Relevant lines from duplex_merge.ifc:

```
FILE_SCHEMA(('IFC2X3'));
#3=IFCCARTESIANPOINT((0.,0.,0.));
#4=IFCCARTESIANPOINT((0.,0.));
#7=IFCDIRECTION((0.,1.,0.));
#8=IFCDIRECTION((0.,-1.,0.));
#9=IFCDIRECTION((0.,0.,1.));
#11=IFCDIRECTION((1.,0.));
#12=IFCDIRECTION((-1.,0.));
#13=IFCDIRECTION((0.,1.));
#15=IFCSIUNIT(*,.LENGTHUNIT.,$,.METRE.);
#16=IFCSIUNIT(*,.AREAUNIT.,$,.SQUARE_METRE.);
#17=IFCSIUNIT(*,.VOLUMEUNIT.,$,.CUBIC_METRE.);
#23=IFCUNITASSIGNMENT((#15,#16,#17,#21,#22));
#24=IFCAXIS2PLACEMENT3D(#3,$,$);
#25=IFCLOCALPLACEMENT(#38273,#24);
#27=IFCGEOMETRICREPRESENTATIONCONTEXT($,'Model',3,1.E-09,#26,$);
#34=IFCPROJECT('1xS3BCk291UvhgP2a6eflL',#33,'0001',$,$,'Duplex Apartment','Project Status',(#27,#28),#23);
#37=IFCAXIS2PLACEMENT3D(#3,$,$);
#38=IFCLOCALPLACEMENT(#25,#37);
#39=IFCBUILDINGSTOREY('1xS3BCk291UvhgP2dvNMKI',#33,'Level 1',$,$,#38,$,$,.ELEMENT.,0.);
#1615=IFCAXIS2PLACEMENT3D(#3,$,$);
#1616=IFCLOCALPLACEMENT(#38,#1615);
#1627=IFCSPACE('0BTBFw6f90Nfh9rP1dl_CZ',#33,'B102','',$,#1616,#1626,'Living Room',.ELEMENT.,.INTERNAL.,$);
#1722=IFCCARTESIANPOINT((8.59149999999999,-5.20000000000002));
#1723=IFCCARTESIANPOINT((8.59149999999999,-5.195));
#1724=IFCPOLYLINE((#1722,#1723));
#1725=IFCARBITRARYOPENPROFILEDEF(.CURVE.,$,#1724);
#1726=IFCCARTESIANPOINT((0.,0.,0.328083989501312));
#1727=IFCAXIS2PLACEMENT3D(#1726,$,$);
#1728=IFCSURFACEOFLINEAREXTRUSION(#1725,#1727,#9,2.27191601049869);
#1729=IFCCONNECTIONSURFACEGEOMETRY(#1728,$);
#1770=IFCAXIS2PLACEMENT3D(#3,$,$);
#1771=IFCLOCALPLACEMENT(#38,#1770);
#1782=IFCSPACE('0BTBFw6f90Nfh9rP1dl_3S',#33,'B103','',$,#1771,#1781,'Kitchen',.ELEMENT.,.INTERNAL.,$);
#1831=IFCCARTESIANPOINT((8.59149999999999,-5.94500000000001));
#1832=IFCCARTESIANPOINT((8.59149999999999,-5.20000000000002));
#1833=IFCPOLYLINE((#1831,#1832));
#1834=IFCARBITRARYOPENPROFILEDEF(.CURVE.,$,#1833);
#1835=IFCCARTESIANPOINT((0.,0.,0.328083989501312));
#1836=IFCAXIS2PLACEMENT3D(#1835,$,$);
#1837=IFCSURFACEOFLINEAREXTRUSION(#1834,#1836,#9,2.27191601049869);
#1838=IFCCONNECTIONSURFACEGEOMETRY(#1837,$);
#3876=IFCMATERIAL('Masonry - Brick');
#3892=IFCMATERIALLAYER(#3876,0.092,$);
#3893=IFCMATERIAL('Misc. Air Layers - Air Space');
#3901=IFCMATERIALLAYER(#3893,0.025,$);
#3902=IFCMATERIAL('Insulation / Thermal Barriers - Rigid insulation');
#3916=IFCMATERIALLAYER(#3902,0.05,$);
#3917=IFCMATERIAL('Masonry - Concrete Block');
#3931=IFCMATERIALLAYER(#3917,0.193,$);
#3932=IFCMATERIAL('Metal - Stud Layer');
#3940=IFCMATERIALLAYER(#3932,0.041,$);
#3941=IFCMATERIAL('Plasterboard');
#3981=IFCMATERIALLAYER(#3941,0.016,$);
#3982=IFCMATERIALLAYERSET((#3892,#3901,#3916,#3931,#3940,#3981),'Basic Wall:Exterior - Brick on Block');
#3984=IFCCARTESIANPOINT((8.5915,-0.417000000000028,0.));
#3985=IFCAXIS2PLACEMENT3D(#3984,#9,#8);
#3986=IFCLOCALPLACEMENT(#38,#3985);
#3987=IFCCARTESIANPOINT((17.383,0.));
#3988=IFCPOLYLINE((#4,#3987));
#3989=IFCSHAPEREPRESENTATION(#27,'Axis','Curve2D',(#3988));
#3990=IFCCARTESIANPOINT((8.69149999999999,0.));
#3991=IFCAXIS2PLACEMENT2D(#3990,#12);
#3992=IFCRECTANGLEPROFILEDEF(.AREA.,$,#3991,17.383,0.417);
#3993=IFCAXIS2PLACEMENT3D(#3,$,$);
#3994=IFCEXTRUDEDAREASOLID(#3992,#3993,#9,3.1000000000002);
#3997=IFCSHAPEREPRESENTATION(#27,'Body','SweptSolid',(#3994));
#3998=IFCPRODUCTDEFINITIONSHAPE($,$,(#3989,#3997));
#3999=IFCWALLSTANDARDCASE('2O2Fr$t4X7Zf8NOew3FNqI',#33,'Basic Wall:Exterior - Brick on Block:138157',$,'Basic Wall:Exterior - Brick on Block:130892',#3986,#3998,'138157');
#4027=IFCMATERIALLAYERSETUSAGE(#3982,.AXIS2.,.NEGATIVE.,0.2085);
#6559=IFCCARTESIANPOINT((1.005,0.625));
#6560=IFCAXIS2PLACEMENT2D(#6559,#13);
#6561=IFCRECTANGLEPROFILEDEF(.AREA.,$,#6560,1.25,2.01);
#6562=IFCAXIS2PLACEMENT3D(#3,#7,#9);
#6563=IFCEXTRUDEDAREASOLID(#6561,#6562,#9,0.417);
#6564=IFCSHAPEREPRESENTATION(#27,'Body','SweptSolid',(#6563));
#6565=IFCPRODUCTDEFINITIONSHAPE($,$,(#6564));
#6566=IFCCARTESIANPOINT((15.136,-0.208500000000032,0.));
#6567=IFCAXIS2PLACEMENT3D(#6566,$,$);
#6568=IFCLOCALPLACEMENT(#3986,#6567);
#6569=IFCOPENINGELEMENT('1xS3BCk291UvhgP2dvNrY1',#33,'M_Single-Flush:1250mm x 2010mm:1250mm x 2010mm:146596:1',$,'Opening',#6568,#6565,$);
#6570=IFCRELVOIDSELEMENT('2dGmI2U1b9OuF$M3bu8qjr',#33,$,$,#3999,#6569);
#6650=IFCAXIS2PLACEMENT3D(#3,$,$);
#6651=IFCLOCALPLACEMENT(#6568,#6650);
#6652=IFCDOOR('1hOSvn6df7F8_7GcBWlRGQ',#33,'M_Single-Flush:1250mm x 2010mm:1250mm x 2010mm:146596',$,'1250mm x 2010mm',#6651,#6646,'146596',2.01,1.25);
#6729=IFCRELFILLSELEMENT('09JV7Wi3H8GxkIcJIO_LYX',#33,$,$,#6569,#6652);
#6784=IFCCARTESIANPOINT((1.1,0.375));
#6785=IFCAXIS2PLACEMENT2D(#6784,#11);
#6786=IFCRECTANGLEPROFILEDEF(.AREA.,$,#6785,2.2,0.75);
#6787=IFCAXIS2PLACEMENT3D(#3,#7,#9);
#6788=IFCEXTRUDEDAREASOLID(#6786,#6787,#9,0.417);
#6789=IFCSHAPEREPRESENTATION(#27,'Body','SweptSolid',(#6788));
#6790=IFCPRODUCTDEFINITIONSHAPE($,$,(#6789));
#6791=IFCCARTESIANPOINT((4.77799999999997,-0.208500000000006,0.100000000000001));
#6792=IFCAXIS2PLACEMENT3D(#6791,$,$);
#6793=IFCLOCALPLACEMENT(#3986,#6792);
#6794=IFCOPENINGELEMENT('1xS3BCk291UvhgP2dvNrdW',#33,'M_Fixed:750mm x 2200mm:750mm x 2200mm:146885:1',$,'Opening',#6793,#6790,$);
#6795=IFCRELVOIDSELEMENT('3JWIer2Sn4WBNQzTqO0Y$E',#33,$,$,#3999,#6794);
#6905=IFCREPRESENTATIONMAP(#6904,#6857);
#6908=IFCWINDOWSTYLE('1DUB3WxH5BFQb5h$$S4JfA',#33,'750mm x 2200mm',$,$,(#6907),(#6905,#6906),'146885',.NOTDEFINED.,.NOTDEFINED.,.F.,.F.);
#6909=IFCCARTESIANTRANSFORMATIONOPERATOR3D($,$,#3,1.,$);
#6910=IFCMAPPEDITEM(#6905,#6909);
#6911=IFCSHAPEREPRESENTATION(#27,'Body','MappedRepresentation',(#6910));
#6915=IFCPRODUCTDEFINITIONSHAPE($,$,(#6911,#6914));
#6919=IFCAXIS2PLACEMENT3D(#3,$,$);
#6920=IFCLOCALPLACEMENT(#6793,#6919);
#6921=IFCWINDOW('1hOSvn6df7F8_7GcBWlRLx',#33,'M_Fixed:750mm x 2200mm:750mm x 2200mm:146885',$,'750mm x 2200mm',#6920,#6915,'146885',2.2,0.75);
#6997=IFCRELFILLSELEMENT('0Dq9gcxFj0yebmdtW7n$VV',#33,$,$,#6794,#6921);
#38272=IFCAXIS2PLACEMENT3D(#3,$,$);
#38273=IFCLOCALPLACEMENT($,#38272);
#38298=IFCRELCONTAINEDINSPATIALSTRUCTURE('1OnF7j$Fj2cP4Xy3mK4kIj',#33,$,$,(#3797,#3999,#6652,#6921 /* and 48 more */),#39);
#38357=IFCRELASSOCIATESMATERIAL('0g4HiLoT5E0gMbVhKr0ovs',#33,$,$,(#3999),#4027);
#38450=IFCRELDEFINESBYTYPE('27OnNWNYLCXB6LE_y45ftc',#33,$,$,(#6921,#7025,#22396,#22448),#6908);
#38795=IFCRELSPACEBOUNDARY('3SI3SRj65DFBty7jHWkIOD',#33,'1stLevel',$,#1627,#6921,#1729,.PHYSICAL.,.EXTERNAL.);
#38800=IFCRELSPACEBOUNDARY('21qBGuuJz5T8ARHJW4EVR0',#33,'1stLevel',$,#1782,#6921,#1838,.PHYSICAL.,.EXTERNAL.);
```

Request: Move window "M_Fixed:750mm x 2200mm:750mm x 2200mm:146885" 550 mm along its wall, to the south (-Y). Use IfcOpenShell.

```python
import numpy as np
import ifcopenshell
import ifcopenshell.api.geometry
import ifcopenshell.util.placement
import ifcopenshell.util.unit

model = ifcopenshell.open("duplex_merge.ifc")
unit_scale = ifcopenshell.util.unit.calculate_unit_scale(model)

window = model.by_guid("1hOSvn6df7F8_7GcBWlRLx")
opening = window.FillsVoids[0].RelatingOpeningElement
wall = opening.VoidsElements[0].RelatingBuildingElement

wall_matrix = ifcopenshell.util.placement.get_local_placement(wall.ObjectPlacement)
shift = wall_matrix[:3, 0] * 0.55 / unit_scale
before = ifcopenshell.util.placement.get_local_placement(window.ObjectPlacement)[:3, 3].copy()

# The window is placed relative to its opening, so it follows when the opening moves.
matrix = ifcopenshell.util.placement.get_local_placement(opening.ObjectPlacement)
matrix[:3, 3] += shift
ifcopenshell.api.geometry.edit_object_placement(
    model, product=opening, matrix=matrix, is_si=False, should_transform_children=True
)

# Space boundary surfaces are stored in each space's coordinates; move them too.
for rel in window.ProvidesBoundaries:
    if not rel.ConnectionGeometry:
        continue
    surface = rel.ConnectionGeometry.SurfaceOnRelatingElement
    space_matrix = ifcopenshell.util.placement.get_local_placement(rel.RelatingSpace.ObjectPlacement)
    point = np.array(surface.Position.Location.Coordinates) + space_matrix[:3, :3].T @ shift
    surface.Position = model.createIfcAxis2Placement3D(
        model.createIfcCartesianPoint(point.tolist()), surface.Position.Axis, surface.Position.RefDirection
    )

after = ifcopenshell.util.placement.get_local_placement(window.ObjectPlacement)[:3, 3]
print("window moved by", (after - before).round(3) + 0.0)

model.write("duplex_merge_v2.ifc")
```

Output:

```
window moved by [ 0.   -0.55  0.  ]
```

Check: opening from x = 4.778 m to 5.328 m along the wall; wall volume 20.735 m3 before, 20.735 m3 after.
